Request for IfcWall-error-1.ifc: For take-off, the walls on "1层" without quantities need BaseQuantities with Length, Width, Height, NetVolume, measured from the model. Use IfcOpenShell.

First a look at what the model holds.

```python
import ifcopenshell
import ifcopenshell.util.element
import ifcopenshell.util.unit

model = ifcopenshell.open("IfcWall-error-1.ifc")
print(model.schema)
for unit_type in ("LENGTHUNIT", "AREAUNIT", "VOLUMEUNIT"):
    print(unit_type, ifcopenshell.util.unit.calculate_unit_scale(model, unit_type))
storey = next(s for s in model.by_type("IfcBuildingStorey") if s.Name == "1层")
walls = [e for e in ifcopenshell.util.element.get_decomposition(storey) if e.is_a("IfcWall")]
for e in sorted(walls, key=lambda e: e.id()):
    print(e.id(), e.is_a(), e.Name, list(ifcopenshell.util.element.get_psets(e, qtos_only=True)), sep=" | ")
```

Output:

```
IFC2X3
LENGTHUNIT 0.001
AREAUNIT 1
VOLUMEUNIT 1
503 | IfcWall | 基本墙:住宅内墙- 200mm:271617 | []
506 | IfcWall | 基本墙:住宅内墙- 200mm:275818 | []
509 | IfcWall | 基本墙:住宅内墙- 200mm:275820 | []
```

```python
import ifcopenshell
import ifcopenshell.api.pset
import ifcopenshell.geom
import ifcopenshell.util.element
import ifcopenshell.util.shape
import ifcopenshell.util.unit

model = ifcopenshell.open("IfcWall-error-1.ifc")
unit_scale = ifcopenshell.util.unit.calculate_unit_scale(model)
volume_scale = ifcopenshell.util.unit.calculate_unit_scale(model, "VOLUMEUNIT")
settings = ifcopenshell.geom.settings()

storey = next(s for s in model.by_type("IfcBuildingStorey") if s.Name == "1层")
walls = [e for e in ifcopenshell.util.element.get_decomposition(storey) if e.is_a("IfcWall")]

for e in sorted(walls, key=lambda e: e.id()):
    if ifcopenshell.util.element.get_psets(e, qtos_only=True, should_inherit=False):
        continue
    # Geometry comes back in metres, in the element's own axes.
    shape = ifcopenshell.geom.create_shape(settings, e)
    values = {
        "Length": ifcopenshell.util.shape.get_x(shape.geometry) / unit_scale,
        "Width": ifcopenshell.util.shape.get_y(shape.geometry) / unit_scale,
        "Height": ifcopenshell.util.shape.get_z(shape.geometry) / unit_scale,
        "NetVolume": ifcopenshell.util.shape.get_volume(shape.geometry) / volume_scale,
    }
    qto = ifcopenshell.api.pset.add_qto(model, product=e, name="BaseQuantities")
    ifcopenshell.api.pset.edit_qto(model, qto=qto, properties=values)
    print(e.id(), {k: round(v, 3) for k, v in values.items()})

model.write("IfcWall-error-1_updated.ifc")
```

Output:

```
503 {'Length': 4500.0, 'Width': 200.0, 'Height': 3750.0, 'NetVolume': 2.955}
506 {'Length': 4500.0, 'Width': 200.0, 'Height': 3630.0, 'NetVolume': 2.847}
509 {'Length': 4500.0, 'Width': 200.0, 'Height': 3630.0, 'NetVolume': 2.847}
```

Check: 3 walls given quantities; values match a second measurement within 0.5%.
